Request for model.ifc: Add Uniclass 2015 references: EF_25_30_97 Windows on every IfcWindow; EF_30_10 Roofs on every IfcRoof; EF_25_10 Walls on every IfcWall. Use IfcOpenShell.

First a look at what the model holds.

```python
import ifcopenshell

model = ifcopenshell.open("model.ifc")
print(model.schema)
print("classifications:", [c.Name for c in model.by_type("IfcClassification")])
for ifc_class in ("IfcDoor", "IfcRoof", "IfcStair", "IfcWall", "IfcWindow"):
    print(ifc_class, len(model.by_type(ifc_class)))
```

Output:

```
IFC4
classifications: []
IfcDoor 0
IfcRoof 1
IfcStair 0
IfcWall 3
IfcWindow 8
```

```python
import ifcopenshell
import ifcopenshell.api.classification

model = ifcopenshell.open("model.ifc")

system = ifcopenshell.api.classification.add_classification(model, classification="Uniclass 2015")

codes = {
    "IfcWindow": ("EF_25_30_97", "Windows"),
    "IfcRoof": ("EF_30_10", "Roofs"),
    "IfcWall": ("EF_25_10", "Walls"),
}
for ifc_class, (code, name) in codes.items():
    products = model.by_type(ifc_class)
    ifcopenshell.api.classification.add_reference(
        model, products=products, classification=system, identification=code, name=name
    )
    print(code, len(products))

model.write("model_v2.ifc")
```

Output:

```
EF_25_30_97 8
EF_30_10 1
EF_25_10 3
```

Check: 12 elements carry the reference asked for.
